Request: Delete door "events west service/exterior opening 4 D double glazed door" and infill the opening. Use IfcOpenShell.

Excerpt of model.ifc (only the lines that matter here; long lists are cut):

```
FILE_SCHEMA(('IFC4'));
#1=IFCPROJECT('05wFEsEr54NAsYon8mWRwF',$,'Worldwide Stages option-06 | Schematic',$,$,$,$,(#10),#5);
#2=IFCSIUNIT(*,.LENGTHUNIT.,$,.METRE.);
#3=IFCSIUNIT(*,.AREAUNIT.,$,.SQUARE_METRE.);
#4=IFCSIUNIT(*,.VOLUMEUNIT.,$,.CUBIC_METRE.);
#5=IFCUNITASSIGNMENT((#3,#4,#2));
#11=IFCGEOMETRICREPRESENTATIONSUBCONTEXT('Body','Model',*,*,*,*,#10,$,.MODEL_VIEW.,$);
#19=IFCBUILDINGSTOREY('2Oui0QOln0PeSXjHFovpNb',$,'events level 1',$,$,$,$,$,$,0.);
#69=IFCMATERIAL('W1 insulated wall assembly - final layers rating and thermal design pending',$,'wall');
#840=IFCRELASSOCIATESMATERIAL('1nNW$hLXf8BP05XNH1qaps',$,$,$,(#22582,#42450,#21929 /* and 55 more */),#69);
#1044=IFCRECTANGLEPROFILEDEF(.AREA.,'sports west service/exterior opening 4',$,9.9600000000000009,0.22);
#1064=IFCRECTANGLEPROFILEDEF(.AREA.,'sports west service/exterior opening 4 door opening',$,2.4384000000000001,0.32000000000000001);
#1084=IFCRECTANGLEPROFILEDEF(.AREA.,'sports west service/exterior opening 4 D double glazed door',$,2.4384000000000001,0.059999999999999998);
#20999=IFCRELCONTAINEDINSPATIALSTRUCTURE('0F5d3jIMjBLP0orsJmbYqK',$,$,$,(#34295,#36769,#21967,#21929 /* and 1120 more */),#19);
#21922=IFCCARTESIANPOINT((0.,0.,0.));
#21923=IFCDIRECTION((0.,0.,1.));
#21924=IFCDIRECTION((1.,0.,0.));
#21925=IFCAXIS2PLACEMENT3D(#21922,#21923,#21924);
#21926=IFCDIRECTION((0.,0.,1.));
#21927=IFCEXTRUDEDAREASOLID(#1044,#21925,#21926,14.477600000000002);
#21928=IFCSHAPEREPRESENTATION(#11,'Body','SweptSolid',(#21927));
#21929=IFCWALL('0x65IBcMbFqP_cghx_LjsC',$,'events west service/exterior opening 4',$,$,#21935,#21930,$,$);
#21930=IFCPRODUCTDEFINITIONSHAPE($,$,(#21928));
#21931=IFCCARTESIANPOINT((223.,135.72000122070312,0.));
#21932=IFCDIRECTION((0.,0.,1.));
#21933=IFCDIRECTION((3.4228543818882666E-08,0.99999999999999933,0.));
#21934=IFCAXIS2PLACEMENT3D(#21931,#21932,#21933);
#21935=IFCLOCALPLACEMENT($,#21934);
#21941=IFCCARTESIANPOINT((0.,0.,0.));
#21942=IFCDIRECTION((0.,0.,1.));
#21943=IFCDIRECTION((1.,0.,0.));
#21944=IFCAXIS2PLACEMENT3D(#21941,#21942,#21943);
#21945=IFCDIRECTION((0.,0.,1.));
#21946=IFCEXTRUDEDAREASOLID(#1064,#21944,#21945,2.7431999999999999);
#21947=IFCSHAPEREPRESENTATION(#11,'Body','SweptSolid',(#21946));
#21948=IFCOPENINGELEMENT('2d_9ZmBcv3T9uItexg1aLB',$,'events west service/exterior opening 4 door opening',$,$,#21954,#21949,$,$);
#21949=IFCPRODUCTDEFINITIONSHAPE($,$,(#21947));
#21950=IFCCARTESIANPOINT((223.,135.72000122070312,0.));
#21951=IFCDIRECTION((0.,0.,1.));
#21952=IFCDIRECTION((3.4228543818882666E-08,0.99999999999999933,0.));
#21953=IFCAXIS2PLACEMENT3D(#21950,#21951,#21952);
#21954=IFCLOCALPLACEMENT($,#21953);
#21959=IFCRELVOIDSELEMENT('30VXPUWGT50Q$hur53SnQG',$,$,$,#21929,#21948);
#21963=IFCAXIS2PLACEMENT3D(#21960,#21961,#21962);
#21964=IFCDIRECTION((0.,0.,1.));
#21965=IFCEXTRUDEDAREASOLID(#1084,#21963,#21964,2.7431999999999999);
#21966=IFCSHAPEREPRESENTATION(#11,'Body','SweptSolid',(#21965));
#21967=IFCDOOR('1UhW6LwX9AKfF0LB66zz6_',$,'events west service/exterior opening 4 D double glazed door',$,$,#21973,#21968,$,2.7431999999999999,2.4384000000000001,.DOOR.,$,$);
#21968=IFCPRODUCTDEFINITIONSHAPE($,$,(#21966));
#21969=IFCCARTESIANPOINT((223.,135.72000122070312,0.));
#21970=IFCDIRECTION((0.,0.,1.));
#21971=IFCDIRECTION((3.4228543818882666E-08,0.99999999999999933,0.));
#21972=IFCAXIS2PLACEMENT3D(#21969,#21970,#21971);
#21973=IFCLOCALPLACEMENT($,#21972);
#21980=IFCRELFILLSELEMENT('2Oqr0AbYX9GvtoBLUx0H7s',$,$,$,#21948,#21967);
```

```python
import ifcopenshell
import ifcopenshell.api.feature
import ifcopenshell.api.root
import ifcopenshell.geom
import ifcopenshell.util.shape

model = ifcopenshell.open("model.ifc")
settings = ifcopenshell.geom.settings()


def volume(element):
    """Net volume in cubic metres, openings subtracted."""
    shape = ifcopenshell.geom.create_shape(settings, element)
    return ifcopenshell.util.shape.get_volume(shape.geometry)


door = model.by_id(21967)
opening = door.FillsVoids[0].RelatingOpeningElement
wall = opening.VoidsElements[0].RelatingBuildingElement
before = volume(wall)

ifcopenshell.api.root.remove_product(model, product=door)
ifcopenshell.api.feature.remove_feature(model, feature=opening)

after = volume(wall)

print(f"wall volume {before:.3f} -> {after:.3f} m3")

model.write("model_v2.ifc")
```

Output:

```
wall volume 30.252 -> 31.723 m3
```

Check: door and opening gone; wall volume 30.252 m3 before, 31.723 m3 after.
